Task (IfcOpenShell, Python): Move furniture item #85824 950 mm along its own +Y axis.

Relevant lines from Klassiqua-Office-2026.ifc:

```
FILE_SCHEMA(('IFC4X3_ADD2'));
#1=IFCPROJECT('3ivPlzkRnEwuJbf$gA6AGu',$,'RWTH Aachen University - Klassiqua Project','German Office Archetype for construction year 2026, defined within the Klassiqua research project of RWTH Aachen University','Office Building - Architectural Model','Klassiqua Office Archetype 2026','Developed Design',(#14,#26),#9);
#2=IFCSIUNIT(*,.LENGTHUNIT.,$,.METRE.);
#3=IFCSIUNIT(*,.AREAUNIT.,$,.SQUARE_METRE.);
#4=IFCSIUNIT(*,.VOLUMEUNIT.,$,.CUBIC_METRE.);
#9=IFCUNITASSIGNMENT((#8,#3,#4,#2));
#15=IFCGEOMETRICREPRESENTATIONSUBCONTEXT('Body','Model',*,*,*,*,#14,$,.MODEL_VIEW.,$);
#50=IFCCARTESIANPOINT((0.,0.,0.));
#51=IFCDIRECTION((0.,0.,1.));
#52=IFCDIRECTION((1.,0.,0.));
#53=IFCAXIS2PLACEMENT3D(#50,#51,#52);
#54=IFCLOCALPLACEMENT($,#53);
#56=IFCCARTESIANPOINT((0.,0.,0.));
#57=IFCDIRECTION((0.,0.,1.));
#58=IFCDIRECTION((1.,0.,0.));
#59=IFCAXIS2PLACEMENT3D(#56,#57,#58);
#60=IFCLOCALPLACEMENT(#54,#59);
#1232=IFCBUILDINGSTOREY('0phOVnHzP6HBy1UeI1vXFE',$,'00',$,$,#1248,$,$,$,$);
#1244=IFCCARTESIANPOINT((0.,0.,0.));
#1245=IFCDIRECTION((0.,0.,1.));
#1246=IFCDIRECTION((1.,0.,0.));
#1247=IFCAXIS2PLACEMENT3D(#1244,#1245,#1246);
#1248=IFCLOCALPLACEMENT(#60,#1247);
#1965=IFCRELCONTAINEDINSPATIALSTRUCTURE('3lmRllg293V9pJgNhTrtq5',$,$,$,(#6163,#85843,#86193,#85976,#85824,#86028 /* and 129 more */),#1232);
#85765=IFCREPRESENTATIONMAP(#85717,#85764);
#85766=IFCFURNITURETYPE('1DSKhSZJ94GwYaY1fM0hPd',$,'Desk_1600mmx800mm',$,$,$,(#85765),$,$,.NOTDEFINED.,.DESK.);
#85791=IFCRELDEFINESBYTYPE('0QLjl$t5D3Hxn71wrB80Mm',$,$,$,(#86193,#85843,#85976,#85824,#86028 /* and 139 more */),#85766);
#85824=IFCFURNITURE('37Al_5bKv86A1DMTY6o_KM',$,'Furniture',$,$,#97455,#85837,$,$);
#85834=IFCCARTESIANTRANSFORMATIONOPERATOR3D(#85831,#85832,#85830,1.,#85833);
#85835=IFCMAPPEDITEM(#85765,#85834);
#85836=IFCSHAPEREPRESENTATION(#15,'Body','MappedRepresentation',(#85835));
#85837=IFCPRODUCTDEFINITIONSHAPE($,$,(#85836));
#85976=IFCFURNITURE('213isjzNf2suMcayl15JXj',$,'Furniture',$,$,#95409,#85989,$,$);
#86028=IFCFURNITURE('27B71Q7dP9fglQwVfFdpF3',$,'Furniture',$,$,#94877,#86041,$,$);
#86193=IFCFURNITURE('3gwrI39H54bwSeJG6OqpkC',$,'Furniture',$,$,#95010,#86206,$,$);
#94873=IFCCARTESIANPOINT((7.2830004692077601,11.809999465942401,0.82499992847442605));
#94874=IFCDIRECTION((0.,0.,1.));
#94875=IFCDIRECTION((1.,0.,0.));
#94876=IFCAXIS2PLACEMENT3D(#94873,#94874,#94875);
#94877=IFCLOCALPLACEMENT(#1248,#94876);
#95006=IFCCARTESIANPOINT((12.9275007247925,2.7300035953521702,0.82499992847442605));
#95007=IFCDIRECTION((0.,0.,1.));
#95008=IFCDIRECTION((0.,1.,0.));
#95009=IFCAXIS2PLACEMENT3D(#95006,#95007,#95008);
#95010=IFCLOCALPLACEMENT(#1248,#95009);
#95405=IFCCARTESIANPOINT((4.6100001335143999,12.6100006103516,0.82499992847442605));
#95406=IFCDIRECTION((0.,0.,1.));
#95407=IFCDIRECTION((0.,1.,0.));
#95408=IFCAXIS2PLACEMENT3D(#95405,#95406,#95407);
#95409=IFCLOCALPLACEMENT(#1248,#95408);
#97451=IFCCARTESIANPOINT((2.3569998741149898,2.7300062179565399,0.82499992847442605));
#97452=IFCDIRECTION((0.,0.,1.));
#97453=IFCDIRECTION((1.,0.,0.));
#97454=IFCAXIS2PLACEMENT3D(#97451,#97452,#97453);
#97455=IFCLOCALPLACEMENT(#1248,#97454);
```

```python
import ifcopenshell
import ifcopenshell.api.geometry
import ifcopenshell.util.placement
import ifcopenshell.util.unit

model = ifcopenshell.open("Klassiqua-Office-2026.ifc")
unit_scale = ifcopenshell.util.unit.calculate_unit_scale(model)

item = model.by_id(85824)
matrix = ifcopenshell.util.placement.get_local_placement(item.ObjectPlacement)
matrix[:3, 3] += matrix[:3, 1] * 0.95 / unit_scale
ifcopenshell.api.geometry.edit_object_placement(model, product=item, matrix=matrix, is_si=False)

print(ifcopenshell.util.placement.get_local_placement(item.ObjectPlacement).round(3) + 0.0)

model.write("Klassiqua-Office-2026_v2.ifc")
```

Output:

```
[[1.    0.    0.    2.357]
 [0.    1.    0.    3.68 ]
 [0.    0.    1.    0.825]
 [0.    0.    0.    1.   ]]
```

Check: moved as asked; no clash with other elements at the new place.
